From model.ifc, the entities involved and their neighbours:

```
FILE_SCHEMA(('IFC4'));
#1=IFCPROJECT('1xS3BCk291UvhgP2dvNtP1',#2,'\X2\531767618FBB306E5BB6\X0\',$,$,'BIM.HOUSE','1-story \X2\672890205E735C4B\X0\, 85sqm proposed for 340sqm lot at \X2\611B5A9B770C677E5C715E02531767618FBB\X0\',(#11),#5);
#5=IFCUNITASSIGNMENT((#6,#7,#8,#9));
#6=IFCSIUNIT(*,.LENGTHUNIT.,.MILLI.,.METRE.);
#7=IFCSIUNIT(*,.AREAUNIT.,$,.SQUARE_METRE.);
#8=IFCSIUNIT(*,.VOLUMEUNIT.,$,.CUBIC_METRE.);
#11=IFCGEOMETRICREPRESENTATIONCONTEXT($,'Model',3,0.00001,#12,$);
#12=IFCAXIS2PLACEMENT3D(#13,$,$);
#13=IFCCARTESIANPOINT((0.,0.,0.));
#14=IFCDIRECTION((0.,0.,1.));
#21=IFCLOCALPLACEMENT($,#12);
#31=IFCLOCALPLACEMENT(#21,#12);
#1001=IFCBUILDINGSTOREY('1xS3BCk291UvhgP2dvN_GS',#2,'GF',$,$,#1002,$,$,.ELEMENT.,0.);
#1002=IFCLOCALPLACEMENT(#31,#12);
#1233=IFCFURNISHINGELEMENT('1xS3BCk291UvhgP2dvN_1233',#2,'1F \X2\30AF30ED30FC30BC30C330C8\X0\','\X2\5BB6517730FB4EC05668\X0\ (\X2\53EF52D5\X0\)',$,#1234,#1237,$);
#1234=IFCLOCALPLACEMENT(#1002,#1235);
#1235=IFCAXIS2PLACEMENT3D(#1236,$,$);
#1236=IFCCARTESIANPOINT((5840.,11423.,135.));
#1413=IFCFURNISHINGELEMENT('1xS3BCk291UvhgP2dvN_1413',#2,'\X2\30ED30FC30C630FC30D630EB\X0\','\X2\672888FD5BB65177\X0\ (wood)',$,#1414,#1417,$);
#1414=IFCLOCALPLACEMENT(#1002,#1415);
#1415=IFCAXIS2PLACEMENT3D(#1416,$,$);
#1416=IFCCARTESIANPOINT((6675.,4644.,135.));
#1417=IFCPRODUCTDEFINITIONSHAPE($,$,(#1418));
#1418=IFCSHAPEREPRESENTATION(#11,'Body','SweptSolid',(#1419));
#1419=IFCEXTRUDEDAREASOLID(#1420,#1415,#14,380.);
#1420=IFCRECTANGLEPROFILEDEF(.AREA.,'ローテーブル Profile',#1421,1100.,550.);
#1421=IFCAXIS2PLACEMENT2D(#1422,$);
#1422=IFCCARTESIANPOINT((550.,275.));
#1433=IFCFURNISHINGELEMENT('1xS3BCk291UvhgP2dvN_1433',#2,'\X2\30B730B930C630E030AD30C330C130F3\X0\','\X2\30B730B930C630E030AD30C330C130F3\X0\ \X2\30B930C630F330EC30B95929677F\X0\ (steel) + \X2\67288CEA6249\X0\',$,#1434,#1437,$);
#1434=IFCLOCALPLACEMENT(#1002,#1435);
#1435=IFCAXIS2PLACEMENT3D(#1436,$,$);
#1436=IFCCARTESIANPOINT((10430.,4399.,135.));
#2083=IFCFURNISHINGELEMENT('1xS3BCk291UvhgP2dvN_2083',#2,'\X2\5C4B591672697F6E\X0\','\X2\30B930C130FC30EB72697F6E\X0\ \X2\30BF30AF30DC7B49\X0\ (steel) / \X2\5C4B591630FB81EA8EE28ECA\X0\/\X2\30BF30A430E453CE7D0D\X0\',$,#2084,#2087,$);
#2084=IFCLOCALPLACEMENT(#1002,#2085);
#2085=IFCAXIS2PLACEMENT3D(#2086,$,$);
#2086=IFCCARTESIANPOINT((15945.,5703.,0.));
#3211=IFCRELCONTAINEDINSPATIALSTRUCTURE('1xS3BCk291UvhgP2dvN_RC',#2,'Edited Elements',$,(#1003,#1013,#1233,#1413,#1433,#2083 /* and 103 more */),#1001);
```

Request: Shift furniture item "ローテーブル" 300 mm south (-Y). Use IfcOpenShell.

```python
import ifcopenshell
import ifcopenshell.api.geometry
import ifcopenshell.util.placement

model = ifcopenshell.open("model.ifc")

item = model.by_id(1413)
matrix = ifcopenshell.util.placement.get_local_placement(item.ObjectPlacement)
matrix[1, 3] -= 300.0
ifcopenshell.api.geometry.edit_object_placement(model, product=item, matrix=matrix, is_si=False)

print(ifcopenshell.util.placement.get_local_placement(item.ObjectPlacement).round(3) + 0.0)

model.write("model_updated.ifc")
```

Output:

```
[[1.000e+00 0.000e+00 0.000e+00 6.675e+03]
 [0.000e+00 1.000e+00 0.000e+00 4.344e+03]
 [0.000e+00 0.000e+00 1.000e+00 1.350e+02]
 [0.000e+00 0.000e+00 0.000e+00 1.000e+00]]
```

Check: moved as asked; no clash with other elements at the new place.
